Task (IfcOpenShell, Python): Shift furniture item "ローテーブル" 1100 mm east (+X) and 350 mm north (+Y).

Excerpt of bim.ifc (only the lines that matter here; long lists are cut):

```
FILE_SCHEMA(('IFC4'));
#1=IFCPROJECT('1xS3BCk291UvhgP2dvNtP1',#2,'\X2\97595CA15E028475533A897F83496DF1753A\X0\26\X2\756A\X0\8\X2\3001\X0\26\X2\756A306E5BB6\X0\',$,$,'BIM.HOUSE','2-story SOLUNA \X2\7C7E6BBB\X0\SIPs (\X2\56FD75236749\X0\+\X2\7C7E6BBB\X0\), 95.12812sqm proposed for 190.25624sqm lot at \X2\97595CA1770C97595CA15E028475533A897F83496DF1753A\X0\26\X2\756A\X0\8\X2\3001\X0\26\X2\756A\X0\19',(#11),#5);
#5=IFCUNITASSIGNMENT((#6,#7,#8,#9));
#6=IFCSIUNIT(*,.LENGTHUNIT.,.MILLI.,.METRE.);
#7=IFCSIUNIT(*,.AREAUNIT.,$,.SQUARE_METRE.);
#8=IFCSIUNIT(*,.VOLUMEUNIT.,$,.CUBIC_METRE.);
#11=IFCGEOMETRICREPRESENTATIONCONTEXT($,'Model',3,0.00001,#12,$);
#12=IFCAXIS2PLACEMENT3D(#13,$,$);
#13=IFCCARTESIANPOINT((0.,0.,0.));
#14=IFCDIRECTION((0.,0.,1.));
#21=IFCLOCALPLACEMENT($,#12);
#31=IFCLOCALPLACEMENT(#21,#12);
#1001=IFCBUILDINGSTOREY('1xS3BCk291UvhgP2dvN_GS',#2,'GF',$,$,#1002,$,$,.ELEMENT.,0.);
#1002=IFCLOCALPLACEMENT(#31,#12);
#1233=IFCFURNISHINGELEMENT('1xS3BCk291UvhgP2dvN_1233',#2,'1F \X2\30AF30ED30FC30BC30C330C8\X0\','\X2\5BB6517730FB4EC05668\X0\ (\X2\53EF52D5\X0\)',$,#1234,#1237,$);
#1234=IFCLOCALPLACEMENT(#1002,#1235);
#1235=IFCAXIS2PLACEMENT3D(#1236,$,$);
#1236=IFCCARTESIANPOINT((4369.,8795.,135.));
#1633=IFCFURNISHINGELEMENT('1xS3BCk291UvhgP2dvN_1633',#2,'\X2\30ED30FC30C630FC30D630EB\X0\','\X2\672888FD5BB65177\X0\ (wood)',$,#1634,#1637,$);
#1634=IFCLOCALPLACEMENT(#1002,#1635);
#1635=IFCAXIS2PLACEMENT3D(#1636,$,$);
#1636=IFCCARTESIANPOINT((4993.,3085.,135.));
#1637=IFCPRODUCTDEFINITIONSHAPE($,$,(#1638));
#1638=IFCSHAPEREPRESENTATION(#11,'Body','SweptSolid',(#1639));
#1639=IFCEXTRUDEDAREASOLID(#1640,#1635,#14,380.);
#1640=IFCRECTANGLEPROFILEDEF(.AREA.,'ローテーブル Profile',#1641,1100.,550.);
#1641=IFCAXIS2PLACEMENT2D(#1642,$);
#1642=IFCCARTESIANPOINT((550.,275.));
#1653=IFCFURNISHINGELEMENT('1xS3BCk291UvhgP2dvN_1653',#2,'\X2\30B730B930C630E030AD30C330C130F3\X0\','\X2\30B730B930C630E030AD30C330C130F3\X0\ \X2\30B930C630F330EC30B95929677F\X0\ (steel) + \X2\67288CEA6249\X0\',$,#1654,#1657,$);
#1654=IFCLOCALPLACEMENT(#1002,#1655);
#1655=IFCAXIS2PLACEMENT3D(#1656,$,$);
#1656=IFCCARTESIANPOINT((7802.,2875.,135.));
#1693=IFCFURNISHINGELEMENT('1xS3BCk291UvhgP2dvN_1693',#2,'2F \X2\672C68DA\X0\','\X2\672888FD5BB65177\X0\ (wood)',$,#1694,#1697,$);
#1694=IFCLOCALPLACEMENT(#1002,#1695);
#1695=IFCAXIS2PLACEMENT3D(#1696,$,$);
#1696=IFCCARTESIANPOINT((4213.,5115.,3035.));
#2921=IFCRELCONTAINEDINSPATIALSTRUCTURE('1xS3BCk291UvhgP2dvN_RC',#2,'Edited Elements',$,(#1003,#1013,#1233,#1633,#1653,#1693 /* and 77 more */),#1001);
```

```python
import ifcopenshell
import ifcopenshell.api.geometry
import ifcopenshell.util.placement

model = ifcopenshell.open("bim.ifc")

item = model.by_guid("1xS3BCk291UvhgP2dvN_1633")
matrix = ifcopenshell.util.placement.get_local_placement(item.ObjectPlacement)
matrix[0, 3] += 1100.0
matrix[1, 3] += 350.0
ifcopenshell.api.geometry.edit_object_placement(model, product=item, matrix=matrix, is_si=False)

print(ifcopenshell.util.placement.get_local_placement(item.ObjectPlacement).round(3) + 0.0)

model.write("bim_updated.ifc")
```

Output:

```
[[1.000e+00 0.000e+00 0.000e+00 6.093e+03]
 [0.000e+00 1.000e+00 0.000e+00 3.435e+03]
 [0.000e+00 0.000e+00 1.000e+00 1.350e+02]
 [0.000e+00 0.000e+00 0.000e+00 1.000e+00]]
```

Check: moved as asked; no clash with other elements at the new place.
